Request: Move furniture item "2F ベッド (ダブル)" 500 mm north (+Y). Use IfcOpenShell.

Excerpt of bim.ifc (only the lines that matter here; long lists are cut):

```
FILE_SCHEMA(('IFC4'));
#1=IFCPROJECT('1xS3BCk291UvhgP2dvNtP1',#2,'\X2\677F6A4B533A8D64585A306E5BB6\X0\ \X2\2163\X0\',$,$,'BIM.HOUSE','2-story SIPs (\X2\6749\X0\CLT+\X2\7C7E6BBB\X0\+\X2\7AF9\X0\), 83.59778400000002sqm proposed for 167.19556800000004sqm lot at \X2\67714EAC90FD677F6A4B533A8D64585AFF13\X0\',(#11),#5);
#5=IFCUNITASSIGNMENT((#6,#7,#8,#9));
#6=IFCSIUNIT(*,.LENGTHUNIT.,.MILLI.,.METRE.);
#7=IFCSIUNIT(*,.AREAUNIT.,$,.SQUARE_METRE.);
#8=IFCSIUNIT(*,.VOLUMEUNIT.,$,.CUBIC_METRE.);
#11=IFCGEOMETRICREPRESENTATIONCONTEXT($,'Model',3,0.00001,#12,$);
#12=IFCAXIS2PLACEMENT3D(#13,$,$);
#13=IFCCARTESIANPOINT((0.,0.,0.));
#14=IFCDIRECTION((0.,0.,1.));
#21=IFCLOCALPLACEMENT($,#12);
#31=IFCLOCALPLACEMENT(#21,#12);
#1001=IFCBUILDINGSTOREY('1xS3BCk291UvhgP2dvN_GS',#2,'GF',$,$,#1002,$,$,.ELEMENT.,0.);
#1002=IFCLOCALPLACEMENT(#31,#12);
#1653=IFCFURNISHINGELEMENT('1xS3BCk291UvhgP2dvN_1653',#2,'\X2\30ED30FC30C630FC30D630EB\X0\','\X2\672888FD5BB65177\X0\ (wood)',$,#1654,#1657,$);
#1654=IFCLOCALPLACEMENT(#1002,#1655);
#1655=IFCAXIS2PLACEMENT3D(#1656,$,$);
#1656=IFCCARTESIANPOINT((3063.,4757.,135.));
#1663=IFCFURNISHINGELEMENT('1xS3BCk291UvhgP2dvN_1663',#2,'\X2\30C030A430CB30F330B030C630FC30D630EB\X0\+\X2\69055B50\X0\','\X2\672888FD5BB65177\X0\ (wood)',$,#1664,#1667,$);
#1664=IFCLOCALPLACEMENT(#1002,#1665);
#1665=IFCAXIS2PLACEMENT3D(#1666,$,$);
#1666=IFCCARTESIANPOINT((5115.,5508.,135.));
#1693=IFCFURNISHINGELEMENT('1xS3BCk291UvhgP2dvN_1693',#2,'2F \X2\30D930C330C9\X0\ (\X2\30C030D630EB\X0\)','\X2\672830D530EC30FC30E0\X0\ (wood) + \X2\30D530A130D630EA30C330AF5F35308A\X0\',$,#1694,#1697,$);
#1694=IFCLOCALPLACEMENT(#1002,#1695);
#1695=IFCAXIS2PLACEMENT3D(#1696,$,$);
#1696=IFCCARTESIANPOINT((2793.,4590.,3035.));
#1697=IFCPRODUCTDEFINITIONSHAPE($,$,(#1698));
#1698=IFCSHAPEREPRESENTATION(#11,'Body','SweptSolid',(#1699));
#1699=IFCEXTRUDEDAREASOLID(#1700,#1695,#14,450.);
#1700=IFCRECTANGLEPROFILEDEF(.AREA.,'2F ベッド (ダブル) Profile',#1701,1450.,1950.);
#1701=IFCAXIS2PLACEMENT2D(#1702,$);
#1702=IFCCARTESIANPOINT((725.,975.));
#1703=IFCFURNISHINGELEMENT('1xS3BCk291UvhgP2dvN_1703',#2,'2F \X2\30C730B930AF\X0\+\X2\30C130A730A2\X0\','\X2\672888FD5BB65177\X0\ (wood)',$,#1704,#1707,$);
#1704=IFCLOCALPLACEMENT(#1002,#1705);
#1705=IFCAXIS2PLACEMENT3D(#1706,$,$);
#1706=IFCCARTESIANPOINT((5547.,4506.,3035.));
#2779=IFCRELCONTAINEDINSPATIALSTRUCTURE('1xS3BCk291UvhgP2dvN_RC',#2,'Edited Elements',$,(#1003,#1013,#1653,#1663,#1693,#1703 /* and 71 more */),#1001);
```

```python
import ifcopenshell
import ifcopenshell.api.geometry
import ifcopenshell.util.placement

model = ifcopenshell.open("bim.ifc")

item = model.by_guid("1xS3BCk291UvhgP2dvN_1693")
matrix = ifcopenshell.util.placement.get_local_placement(item.ObjectPlacement)
matrix[1, 3] += 500.0
ifcopenshell.api.geometry.edit_object_placement(model, product=item, matrix=matrix, is_si=False)

print(ifcopenshell.util.placement.get_local_placement(item.ObjectPlacement).round(3) + 0.0)

model.write("bim_edited.ifc")
```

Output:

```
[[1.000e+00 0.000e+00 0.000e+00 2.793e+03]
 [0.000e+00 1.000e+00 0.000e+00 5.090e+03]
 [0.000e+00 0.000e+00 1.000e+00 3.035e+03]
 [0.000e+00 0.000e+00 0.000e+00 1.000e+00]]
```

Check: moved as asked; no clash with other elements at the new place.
